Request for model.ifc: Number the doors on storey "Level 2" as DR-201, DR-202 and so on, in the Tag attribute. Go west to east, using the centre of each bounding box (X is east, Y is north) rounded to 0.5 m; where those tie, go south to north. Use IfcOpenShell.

First a look at what the model holds.

```python
import ifcopenshell
import ifcopenshell.util.element
import ifcopenshell.util.placement

model = ifcopenshell.open("model.ifc")
print(model.schema)
storey = next(s for s in model.by_type("IfcBuildingStorey") if s.Name == "Level 2")
doors = [e for e in ifcopenshell.util.element.get_decomposition(storey) if e.is_a("IfcDoor")]
for e in sorted(doors, key=lambda e: e.id()):
    origin = ifcopenshell.util.placement.get_local_placement(e.ObjectPlacement)[:3, 3]
    print(e.id(), e.Tag, e.Name, origin.round(2) + 0.0, sep=" | ")
```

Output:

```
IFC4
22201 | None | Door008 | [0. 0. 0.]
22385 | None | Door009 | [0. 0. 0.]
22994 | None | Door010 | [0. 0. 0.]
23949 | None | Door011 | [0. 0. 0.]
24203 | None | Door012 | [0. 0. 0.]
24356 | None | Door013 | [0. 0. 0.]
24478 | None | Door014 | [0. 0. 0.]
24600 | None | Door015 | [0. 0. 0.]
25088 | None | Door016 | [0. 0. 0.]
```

```python
import ifcopenshell
import ifcopenshell.geom
import ifcopenshell.util.element
import ifcopenshell.util.shape

model = ifcopenshell.open("model.ifc")
settings = ifcopenshell.geom.settings()
settings.set("use-world-coords", True)


def centre(element):
    shape = ifcopenshell.geom.create_shape(settings, element)
    return ifcopenshell.util.shape.get_bbox_centroid(shape.geometry)


storey = next(s for s in model.by_type("IfcBuildingStorey") if s.Name == "Level 2")
doors = [e for e in ifcopenshell.util.element.get_decomposition(storey) if e.is_a("IfcDoor")]

# Insertion points can sit at a corner or the storey origin, so sort by the geometry (in metres).
centres = {e: centre(e) for e in doors}
doors.sort(key=lambda e: (round(centres[e][0] / 0.5), centres[e][1]))

for i, e in enumerate(doors, start=1):
    number = f"DR-2{i:02d}"
    e.Tag = number
    print(e.id(), number)

model.write("model_v2.ifc")
```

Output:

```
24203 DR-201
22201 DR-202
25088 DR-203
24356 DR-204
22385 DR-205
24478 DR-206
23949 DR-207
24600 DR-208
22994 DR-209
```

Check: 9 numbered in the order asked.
